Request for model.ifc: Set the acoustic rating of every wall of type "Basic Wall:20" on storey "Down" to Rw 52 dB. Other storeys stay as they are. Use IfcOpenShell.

First a look at what the model holds.

```python
import ifcopenshell
import ifcopenshell.util.element

model = ifcopenshell.open("model.ifc")
print(model.schema)
storey = next(s for s in model.by_type("IfcBuildingStorey") if s.Name == "Down")
walls = [e for e in ifcopenshell.util.element.get_decomposition(storey) if e.is_a("IfcWall")]
seen = {}
for e in walls:
    element_type = ifcopenshell.util.element.get_type(e)
    key = (element_type.Name if element_type != e and element_type else None, ifcopenshell.util.element.get_pset(e, "Pset_WallCommon", "AcousticRating"))
    seen[key] = seen.get(key, 0) + 1
for (name, value), count in sorted(seen.items(), key=str):
    print(count, "x", name, "|", value)
```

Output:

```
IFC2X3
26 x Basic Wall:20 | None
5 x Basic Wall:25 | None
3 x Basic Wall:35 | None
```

```python
import ifcopenshell
import ifcopenshell.api.pset
import ifcopenshell.util.element

model = ifcopenshell.open("model.ifc")

storey = next(s for s in model.by_type("IfcBuildingStorey") if s.Name == "Down")
walls = [e for e in ifcopenshell.util.element.get_decomposition(storey) if e.is_a("IfcWall")]

count = 0
for e in walls:
    element_type = ifcopenshell.util.element.get_type(e)
    if element_type in (None, e) or element_type.Name != "Basic Wall:20":
        continue
    # add_pset returns the element's existing set when there is one.
    pset = ifcopenshell.api.pset.add_pset(model, product=e, name="Pset_WallCommon")
    ifcopenshell.api.pset.edit_pset(model, pset=pset, properties={"AcousticRating": "Rw 52 dB"})
    count += 1

print(count, "walls updated")

model.write("model_rev.ifc")
```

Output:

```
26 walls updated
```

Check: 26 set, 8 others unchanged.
